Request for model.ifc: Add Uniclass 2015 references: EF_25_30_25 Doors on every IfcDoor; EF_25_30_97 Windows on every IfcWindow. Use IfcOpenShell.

First a look at what the model holds.

```python
import ifcopenshell

model = ifcopenshell.open("model.ifc")
print(model.schema)
print("classifications:", [c.Name for c in model.by_type("IfcClassification")])
for ifc_class in ("IfcDoor", "IfcRoof", "IfcStair", "IfcWall", "IfcWindow"):
    print(ifc_class, len(model.by_type(ifc_class)))
```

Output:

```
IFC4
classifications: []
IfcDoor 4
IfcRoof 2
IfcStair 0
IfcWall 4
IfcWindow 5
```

```python
import ifcopenshell
import ifcopenshell.api.classification

model = ifcopenshell.open("model.ifc")

system = ifcopenshell.api.classification.add_classification(model, classification="Uniclass 2015")

codes = {
    "IfcDoor": ("EF_25_30_25", "Doors"),
    "IfcWindow": ("EF_25_30_97", "Windows"),
}
for ifc_class, (code, name) in codes.items():
    products = model.by_type(ifc_class)
    ifcopenshell.api.classification.add_reference(
        model, products=products, classification=system, identification=code, name=name
    )
    print(code, len(products))

model.write("model_edited.ifc")
```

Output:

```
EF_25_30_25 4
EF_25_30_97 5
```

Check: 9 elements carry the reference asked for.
